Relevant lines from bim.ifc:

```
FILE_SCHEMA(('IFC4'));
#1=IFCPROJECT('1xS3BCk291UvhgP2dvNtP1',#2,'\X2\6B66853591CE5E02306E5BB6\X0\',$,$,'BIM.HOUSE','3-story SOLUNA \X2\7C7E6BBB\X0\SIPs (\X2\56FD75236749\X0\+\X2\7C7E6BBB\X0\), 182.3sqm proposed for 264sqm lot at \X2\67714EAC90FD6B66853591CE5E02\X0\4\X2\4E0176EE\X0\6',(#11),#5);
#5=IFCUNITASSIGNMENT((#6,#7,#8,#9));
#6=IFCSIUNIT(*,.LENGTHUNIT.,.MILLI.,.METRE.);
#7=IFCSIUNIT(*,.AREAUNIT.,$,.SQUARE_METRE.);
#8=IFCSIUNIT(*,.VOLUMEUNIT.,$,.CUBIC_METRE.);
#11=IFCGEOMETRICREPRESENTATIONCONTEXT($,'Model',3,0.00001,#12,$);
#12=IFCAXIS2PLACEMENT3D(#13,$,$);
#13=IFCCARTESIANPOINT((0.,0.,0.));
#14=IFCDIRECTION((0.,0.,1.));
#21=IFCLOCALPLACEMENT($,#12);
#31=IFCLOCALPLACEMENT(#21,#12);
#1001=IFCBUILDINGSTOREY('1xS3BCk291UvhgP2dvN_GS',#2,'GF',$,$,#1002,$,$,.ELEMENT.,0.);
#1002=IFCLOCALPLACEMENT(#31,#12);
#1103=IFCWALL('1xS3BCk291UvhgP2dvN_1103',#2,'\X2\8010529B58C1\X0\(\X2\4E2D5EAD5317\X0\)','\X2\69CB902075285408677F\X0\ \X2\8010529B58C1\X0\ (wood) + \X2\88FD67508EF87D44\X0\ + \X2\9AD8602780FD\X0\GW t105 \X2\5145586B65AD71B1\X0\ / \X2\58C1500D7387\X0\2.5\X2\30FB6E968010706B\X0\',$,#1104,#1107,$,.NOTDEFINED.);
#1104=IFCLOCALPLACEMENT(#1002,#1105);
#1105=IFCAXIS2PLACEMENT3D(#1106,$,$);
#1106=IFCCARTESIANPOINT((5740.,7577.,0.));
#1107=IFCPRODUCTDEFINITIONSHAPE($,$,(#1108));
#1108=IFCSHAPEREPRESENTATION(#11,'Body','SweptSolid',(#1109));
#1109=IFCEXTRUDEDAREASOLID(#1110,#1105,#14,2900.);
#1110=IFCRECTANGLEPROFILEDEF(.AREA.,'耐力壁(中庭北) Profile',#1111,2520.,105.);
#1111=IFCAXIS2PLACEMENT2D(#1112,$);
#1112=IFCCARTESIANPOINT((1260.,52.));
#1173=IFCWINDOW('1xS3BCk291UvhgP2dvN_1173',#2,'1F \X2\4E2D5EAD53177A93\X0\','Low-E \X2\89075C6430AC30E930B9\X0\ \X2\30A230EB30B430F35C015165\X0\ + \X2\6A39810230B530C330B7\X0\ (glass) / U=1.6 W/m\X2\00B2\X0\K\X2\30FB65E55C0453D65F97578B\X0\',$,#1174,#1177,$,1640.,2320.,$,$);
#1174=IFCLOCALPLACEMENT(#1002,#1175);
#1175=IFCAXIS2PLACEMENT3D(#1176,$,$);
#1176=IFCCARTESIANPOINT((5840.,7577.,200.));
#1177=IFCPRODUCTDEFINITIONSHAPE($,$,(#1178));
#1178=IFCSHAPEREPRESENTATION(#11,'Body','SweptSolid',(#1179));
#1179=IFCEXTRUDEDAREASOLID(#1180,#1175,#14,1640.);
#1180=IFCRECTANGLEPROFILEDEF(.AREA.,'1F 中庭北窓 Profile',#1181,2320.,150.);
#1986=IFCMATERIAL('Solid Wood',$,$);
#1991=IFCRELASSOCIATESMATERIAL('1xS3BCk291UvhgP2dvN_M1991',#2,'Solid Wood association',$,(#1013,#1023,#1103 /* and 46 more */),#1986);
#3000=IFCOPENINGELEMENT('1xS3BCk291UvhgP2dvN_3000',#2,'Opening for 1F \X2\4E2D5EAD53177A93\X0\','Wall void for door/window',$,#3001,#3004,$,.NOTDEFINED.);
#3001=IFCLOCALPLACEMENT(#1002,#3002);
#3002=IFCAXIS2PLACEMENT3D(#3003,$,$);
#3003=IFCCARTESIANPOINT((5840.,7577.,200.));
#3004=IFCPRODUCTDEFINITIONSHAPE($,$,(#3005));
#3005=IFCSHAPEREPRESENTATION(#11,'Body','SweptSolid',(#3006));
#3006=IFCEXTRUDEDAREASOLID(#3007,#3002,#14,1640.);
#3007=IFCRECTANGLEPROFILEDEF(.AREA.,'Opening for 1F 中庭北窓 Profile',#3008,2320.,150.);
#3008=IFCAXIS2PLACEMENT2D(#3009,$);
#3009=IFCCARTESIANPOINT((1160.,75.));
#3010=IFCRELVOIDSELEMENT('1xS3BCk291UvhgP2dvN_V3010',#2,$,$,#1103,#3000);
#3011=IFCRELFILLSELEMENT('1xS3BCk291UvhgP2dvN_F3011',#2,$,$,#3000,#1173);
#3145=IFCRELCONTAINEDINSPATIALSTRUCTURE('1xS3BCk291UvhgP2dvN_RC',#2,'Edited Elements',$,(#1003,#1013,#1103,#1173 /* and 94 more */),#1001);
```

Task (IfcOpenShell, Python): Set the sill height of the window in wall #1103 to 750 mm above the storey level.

```python
import numpy as np
import ifcopenshell
import ifcopenshell.api.geometry
import ifcopenshell.geom
import ifcopenshell.util.element
import ifcopenshell.util.placement
import ifcopenshell.util.shape
import ifcopenshell.util.unit

model = ifcopenshell.open("bim.ifc")
unit_scale = ifcopenshell.util.unit.calculate_unit_scale(model)

window = model.by_guid("1xS3BCk291UvhgP2dvN_1173")
opening = window.FillsVoids[0].RelatingOpeningElement
storey = ifcopenshell.util.element.get_container(window, ifc_class="IfcBuildingStorey")
level = ifcopenshell.util.placement.get_local_placement(storey.ObjectPlacement)[2, 3]

# The opening's origin need not be at the sill, so measure its lowest point.
shape = ifcopenshell.geom.create_shape(ifcopenshell.geom.settings(), opening)
bottom = ifcopenshell.util.shape.get_shape_bottom_elevation(shape, shape.geometry) / unit_scale
dz = level + 0.75 / unit_scale - bottom

shift = np.array([0.0, 0.0, dz])
# The window is not placed relative to its opening, so move both.
for product in (opening, window):
    matrix = ifcopenshell.util.placement.get_local_placement(product.ObjectPlacement)
    matrix[:3, 3] += shift
    ifcopenshell.api.geometry.edit_object_placement(model, product=product, matrix=matrix, is_si=False)

print(f"moved by {dz * unit_scale:+.3f} m")

model.write("bim_updated.ifc")
```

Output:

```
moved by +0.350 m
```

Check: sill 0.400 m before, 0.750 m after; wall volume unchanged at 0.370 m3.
